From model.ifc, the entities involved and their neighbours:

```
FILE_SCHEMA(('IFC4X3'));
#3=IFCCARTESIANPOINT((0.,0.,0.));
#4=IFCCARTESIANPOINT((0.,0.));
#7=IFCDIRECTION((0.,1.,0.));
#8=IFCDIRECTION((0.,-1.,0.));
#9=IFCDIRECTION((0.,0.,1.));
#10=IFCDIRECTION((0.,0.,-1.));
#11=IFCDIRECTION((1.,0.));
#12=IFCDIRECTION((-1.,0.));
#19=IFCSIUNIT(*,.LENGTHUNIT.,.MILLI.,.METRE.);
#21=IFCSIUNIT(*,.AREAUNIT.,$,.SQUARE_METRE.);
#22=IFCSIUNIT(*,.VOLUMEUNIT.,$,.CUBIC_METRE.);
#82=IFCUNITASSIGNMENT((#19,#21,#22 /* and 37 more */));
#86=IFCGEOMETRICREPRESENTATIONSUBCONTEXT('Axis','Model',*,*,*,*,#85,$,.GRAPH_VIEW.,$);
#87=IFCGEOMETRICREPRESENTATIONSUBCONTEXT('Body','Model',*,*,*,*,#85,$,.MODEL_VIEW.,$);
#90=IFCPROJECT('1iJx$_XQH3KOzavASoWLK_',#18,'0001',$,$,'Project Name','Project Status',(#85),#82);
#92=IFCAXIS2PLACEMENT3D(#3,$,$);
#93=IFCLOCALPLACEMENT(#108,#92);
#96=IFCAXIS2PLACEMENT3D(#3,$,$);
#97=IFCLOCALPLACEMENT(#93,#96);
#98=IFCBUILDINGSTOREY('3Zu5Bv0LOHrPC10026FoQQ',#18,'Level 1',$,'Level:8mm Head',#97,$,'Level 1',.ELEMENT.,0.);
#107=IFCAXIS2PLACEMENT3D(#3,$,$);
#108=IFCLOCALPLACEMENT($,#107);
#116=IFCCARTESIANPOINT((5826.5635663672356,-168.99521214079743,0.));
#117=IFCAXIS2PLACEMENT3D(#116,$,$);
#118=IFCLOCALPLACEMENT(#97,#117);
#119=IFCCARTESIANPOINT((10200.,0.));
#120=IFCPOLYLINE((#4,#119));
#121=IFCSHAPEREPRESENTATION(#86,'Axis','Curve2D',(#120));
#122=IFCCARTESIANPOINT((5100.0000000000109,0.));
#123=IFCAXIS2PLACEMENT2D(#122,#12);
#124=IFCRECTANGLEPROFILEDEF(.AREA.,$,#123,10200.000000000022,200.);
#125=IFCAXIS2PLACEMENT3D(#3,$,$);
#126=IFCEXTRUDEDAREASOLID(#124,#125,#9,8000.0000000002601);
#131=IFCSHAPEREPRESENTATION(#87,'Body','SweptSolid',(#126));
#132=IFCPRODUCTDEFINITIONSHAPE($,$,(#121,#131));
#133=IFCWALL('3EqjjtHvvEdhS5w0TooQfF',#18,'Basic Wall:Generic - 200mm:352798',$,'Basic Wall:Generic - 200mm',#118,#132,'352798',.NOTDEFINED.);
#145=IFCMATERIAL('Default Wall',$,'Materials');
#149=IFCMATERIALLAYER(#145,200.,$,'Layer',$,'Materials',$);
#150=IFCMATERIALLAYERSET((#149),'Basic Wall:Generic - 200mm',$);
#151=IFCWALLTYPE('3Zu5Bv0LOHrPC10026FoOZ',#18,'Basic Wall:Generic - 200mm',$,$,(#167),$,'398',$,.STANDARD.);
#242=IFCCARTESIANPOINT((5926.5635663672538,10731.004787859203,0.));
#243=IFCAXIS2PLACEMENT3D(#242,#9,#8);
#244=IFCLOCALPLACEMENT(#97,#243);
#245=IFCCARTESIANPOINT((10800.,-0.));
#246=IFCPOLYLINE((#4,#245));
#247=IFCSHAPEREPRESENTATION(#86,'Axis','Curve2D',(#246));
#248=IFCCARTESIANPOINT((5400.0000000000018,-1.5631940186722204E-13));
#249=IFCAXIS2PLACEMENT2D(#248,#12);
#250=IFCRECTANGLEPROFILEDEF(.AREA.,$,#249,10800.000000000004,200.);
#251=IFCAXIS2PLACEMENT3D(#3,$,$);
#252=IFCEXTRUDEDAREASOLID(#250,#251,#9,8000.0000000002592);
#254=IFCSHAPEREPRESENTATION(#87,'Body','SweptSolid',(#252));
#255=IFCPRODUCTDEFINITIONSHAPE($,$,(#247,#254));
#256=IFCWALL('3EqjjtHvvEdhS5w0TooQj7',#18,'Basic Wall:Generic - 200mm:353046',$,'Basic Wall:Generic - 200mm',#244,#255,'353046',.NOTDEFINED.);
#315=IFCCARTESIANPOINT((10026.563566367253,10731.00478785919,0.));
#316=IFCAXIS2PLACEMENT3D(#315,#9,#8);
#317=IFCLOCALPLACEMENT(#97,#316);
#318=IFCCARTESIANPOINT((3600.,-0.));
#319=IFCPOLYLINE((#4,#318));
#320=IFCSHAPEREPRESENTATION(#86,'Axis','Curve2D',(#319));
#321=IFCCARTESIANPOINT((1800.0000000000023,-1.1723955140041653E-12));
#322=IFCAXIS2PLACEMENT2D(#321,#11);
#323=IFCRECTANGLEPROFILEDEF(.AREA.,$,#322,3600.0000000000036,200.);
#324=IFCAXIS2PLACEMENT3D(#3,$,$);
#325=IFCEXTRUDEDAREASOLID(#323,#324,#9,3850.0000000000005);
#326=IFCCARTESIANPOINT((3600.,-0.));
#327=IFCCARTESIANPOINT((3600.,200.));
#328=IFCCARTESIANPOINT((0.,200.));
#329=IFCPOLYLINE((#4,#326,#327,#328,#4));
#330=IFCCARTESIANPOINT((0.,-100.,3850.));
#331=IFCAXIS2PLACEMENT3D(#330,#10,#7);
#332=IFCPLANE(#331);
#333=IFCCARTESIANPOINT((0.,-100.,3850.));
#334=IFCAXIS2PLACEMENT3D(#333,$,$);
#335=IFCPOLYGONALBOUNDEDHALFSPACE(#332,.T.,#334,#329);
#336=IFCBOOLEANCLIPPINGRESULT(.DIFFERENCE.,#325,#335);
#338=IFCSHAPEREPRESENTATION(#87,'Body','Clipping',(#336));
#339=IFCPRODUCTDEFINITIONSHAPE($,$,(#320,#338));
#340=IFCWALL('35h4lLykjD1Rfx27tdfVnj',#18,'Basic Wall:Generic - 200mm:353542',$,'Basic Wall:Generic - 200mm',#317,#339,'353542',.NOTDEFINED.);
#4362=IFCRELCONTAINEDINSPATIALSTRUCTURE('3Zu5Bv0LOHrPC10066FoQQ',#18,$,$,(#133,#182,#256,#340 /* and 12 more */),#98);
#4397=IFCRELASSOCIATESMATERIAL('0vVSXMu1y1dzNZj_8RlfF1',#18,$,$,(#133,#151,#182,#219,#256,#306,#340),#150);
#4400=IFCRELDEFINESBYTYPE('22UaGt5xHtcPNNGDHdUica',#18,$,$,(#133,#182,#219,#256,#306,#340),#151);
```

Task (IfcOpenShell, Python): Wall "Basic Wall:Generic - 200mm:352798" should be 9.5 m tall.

```python
import ifcopenshell
import ifcopenshell.geom
import ifcopenshell.util.representation
import ifcopenshell.util.shape

model = ifcopenshell.open("model.ifc")
settings = ifcopenshell.geom.settings()


def volume(element):
    """Net volume in cubic metres, openings subtracted."""
    shape = ifcopenshell.geom.create_shape(settings, element)
    return ifcopenshell.util.shape.get_volume(shape.geometry)


wall = model.by_guid("3EqjjtHvvEdhS5w0TooQfF")
before = volume(wall)

body = ifcopenshell.util.representation.get_representation(wall, "Model", "Body")
solid = body.Items[0]
old_height = solid.Depth
solid.Depth = 9500.0
after = volume(wall)

print(f"height {old_height:g} -> {solid.Depth:g}, volume {before:.3f} -> {after:.3f} m3")

model.write("model_v2.ifc")
```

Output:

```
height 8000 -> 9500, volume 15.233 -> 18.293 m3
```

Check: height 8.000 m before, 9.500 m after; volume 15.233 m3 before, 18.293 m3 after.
